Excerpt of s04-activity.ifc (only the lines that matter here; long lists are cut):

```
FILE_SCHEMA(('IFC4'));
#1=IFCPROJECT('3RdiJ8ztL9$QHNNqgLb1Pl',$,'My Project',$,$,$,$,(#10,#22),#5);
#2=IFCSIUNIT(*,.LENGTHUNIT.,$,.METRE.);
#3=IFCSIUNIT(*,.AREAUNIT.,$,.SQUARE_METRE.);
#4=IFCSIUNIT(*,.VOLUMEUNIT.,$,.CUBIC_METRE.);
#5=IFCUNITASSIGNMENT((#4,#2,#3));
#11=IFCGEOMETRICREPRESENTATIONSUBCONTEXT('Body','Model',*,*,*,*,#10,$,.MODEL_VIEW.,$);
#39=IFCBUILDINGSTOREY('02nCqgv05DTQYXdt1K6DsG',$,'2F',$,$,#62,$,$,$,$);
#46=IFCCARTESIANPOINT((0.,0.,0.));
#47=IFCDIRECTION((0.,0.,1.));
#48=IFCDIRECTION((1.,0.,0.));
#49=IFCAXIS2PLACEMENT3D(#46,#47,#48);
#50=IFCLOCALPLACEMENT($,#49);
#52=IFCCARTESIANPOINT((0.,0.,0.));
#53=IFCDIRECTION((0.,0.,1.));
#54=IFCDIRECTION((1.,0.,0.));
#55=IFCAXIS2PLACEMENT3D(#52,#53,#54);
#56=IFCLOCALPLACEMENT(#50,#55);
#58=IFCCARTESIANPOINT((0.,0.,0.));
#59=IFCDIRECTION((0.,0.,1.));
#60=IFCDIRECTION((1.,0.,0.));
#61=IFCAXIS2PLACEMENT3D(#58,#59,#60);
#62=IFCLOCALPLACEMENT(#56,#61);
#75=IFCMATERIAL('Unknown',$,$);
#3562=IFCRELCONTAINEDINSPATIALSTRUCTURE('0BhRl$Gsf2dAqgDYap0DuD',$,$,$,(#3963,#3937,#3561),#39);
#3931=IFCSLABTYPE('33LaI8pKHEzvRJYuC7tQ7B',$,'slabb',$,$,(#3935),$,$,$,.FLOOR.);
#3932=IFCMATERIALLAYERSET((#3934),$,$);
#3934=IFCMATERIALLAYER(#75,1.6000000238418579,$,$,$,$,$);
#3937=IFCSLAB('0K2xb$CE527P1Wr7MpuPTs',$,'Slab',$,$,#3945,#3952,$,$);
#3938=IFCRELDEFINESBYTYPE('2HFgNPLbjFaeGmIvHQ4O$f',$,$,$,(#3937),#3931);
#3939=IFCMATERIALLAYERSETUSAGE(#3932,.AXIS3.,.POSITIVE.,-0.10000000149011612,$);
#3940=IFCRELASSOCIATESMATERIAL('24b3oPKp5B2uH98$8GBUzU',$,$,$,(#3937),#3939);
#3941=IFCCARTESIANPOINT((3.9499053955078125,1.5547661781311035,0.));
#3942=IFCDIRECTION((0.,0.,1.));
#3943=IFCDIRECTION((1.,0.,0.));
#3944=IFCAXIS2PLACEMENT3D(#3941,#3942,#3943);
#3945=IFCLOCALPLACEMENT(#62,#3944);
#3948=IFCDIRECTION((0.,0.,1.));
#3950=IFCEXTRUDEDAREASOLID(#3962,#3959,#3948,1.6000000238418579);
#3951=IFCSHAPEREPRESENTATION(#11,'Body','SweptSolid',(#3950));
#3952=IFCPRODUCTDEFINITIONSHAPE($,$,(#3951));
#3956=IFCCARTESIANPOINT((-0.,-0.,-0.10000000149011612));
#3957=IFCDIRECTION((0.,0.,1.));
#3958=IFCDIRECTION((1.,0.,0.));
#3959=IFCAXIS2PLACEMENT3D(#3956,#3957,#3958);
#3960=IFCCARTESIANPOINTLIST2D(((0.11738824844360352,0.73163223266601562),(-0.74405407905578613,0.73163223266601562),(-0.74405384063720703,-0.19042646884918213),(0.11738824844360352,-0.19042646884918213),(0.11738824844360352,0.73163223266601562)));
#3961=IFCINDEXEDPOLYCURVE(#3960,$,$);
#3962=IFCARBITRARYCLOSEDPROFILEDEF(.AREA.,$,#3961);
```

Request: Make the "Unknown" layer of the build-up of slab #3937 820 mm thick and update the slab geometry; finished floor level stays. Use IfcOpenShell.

```python
import ifcopenshell
import ifcopenshell.util.element
import ifcopenshell.util.representation
import ifcopenshell.util.unit

model = ifcopenshell.open("s04-activity.ifc")
unit_scale = ifcopenshell.util.unit.calculate_unit_scale(model)

layer_set = model.by_id(3932)
layer = next(l for l in layer_set.MaterialLayers if l.Material and l.Material.Name == "Unknown")
change = 0.82 / unit_scale - layer.LayerThickness
layer.LayerThickness += change

# Geometry does not follow the layer set by itself.
slabs = [e for e in ifcopenshell.util.element.get_elements_by_material(model, layer_set) if e.is_a("IfcSlab")]
for slab in sorted(slabs, key=lambda e: e.id()):
    body = ifcopenshell.util.representation.get_representation(slab, "Model", "Body")
    solid = body.Items[0]
    old_depth = solid.Depth
    solid.Depth += change
    # Extruded upwards: lower the start of the extrusion so the top stays.
    x, y, z = solid.Position.Location.Coordinates
    solid.Position.Location = model.createIfcCartesianPoint((x, y, z - change))
    print(slab.id(), f"{old_depth:g} -> {solid.Depth:g}")

# The layers are counted up from the underside, which has moved.
for usage in {ifcopenshell.util.element.get_material(slab) for slab in slabs}:
    usage.OffsetFromReferenceLine -= change

model.write("s04-activity_rev.ifc")
```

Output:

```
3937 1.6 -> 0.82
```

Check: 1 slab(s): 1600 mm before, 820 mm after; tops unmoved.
